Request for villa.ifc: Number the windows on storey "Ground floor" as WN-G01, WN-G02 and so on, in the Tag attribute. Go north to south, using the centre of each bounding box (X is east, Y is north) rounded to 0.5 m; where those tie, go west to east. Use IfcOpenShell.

First a look at what the model holds.

```python
import ifcopenshell
import ifcopenshell.util.element
import ifcopenshell.util.placement

model = ifcopenshell.open("villa.ifc")
print(model.schema)
storey = next(s for s in model.by_type("IfcBuildingStorey") if s.Name == "Ground floor")
windows = [e for e in ifcopenshell.util.element.get_decomposition(storey) if e.is_a("IfcWindow")]
for e in sorted(windows, key=lambda e: e.id()):
    origin = ifcopenshell.util.placement.get_local_placement(e.ObjectPlacement)[:3, 3]
    print(e.id(), e.Tag, e.Name, origin.round(2) + 0.0, sep=" | ")
```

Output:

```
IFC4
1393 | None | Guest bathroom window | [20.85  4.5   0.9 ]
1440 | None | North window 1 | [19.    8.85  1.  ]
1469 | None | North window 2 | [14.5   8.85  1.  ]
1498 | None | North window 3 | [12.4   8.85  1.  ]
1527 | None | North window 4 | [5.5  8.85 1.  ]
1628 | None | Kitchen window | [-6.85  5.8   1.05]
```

```python
import ifcopenshell
import ifcopenshell.geom
import ifcopenshell.util.element
import ifcopenshell.util.shape

model = ifcopenshell.open("villa.ifc")
settings = ifcopenshell.geom.settings()
settings.set("use-world-coords", True)


def centre(element):
    shape = ifcopenshell.geom.create_shape(settings, element)
    return ifcopenshell.util.shape.get_bbox_centroid(shape.geometry)


storey = next(s for s in model.by_type("IfcBuildingStorey") if s.Name == "Ground floor")
windows = [e for e in ifcopenshell.util.element.get_decomposition(storey) if e.is_a("IfcWindow")]

# Insertion points can sit at a corner or the storey origin, so sort by the geometry (in metres).
centres = {e: centre(e) for e in windows}
windows.sort(key=lambda e: (-round(centres[e][1] / 0.5), centres[e][0]))

for i, e in enumerate(windows, start=1):
    number = f"WN-G{i:02d}"
    e.Tag = number
    print(e.id(), number)

model.write("villa_v2.ifc")
```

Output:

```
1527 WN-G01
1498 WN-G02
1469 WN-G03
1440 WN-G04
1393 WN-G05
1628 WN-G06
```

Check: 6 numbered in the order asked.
